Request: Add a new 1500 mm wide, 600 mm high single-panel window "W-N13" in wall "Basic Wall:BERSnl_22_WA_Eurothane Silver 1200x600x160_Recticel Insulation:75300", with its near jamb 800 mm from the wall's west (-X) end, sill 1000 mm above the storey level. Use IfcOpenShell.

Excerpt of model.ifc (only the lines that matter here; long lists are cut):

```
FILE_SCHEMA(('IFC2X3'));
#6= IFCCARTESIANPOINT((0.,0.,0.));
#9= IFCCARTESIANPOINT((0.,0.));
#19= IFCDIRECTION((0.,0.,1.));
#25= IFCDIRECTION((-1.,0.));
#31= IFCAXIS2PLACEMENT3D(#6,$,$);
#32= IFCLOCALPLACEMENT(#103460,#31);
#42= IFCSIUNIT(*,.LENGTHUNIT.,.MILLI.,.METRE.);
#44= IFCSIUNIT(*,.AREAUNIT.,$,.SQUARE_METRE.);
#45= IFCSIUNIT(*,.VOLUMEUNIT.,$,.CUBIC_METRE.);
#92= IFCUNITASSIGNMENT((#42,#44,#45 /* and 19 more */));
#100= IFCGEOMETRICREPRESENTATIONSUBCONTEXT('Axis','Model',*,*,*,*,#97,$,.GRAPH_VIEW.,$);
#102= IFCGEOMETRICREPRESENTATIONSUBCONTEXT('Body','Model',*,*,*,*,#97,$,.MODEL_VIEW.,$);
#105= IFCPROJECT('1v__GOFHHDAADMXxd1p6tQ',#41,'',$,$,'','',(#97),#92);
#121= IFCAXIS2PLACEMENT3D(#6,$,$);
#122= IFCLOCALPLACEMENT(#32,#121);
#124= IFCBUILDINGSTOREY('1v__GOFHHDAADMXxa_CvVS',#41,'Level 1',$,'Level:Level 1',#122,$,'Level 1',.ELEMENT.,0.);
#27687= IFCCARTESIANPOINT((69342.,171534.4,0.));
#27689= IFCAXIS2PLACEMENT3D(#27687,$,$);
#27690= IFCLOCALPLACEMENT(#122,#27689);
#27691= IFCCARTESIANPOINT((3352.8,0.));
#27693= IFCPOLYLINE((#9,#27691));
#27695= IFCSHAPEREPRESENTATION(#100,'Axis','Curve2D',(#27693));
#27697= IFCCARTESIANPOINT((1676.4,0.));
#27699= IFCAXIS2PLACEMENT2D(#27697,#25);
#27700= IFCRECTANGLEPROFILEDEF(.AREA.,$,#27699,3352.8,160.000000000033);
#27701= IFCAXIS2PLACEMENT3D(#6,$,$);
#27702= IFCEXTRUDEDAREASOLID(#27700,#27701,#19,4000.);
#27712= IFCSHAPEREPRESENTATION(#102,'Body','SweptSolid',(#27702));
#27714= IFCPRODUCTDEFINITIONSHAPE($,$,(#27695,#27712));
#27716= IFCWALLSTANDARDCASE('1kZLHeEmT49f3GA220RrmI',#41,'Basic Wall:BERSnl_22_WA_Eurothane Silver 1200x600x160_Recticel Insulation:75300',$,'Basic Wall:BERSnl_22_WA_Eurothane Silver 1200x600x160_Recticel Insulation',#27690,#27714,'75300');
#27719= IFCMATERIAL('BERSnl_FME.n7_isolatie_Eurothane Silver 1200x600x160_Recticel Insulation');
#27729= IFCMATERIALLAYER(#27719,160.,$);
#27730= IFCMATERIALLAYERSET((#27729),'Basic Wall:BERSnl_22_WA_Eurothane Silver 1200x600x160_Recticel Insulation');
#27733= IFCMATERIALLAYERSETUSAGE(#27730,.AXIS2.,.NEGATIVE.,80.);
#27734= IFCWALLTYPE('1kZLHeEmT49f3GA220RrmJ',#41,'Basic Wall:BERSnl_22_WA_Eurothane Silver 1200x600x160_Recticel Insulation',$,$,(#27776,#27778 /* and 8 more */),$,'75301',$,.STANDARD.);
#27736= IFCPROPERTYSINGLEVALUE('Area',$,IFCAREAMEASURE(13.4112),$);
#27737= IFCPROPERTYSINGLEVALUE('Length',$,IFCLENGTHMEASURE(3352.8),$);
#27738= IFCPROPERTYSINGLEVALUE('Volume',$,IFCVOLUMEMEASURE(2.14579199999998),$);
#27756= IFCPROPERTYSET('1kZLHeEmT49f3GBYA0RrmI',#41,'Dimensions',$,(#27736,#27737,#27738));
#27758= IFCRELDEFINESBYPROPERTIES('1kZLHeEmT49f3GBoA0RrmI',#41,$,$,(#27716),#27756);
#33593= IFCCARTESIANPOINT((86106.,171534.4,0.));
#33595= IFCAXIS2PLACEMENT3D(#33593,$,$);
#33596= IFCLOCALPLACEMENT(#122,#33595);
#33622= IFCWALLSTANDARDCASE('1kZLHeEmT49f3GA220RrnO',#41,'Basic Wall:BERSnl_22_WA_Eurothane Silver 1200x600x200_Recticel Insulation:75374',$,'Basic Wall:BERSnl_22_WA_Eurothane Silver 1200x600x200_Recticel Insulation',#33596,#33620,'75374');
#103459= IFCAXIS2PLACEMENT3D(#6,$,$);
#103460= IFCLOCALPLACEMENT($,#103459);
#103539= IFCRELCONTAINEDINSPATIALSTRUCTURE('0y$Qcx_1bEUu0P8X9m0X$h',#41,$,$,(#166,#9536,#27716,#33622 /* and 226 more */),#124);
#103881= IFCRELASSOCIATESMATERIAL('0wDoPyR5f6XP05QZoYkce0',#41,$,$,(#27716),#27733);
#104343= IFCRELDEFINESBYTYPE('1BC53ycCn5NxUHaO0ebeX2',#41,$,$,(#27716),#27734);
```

```python
import numpy as np
import ifcopenshell
import ifcopenshell.api.feature
import ifcopenshell.api.geometry
import ifcopenshell.api.pset
import ifcopenshell.api.root
import ifcopenshell.api.spatial
import ifcopenshell.api.type
import ifcopenshell.geom
import ifcopenshell.util.element
import ifcopenshell.util.placement
import ifcopenshell.util.representation
import ifcopenshell.util.shape
import ifcopenshell.util.unit

model = ifcopenshell.open("model.ifc")
unit_scale = ifcopenshell.util.unit.calculate_unit_scale(model)
area_scale = ifcopenshell.util.unit.calculate_unit_scale(model, "AREAUNIT")
volume_scale = ifcopenshell.util.unit.calculate_unit_scale(model, "VOLUMEUNIT")
settings = ifcopenshell.geom.settings()


def volume(element):
    """Net volume in cubic metres, openings subtracted."""
    shape = ifcopenshell.geom.create_shape(settings, element)
    return ifcopenshell.util.shape.get_volume(shape.geometry)


wall = model.by_guid("1kZLHeEmT49f3GA220RrmI")
storey = ifcopenshell.util.element.get_container(wall, ifc_class="IfcBuildingStorey")
context = ifcopenshell.util.representation.get_context(model, "Model", "Body", "MODEL_VIEW")
before = volume(wall)

width, height, from_end, sill = 1.5, 0.6, 0.8, 1  # metres

# The wall runs along its own X axis, and the end named is its -X end.
wall_shape = ifcopenshell.geom.create_shape(settings, wall)
x, y, z = ifcopenshell.util.shape.get_vertices(wall_shape.geometry).T
start = x.min() + from_end
face, thickness = float(y.min()), float(y.max() - y.min())
wall_matrix = ifcopenshell.util.placement.get_local_placement(wall.ObjectPlacement)
level = ifcopenshell.util.placement.get_local_placement(storey.ObjectPlacement)[2, 3]


def in_wall(x, y):
    """Placement at x, y metres in the wall's axes, at sill height."""
    matrix = wall_matrix.copy()
    matrix[:, 3] = wall_matrix @ np.array([x / unit_scale, y / unit_scale, 0.0, 1.0])
    matrix[2, 3] = level + sill / unit_scale
    return matrix


# Opening: a box that overshoots both wall faces by 50 mm.
opening = ifcopenshell.api.root.create_entity(model, ifc_class="IfcOpeningElement")
box = ifcopenshell.api.geometry.add_wall_representation(
    model, context=context, length=width, height=height, thickness=thickness + 0.1
)
ifcopenshell.api.geometry.assign_representation(model, product=opening, representation=box)
ifcopenshell.api.geometry.edit_object_placement(model, product=opening, matrix=in_wall(start, face - 0.05), is_si=False)
ifcopenshell.api.feature.add_feature(model, feature=opening, element=wall)

window = ifcopenshell.api.root.create_entity(model, ifc_class="IfcWindow", name="W-N13")
window.OverallWidth, window.OverallHeight = width / unit_scale, height / unit_scale
body = ifcopenshell.api.geometry.add_window_representation(
    model,
    context=context,
    overall_width=window.OverallWidth,
    overall_height=window.OverallHeight,
    partition_type="SINGLE_PANEL",
)
ifcopenshell.api.geometry.assign_representation(model, product=window, representation=body)
ifcopenshell.api.spatial.assign_container(model, products=[window], relating_structure=storey)
fills = ifcopenshell.api.feature.add_filling(model, opening=opening, element=window)
fills.OwnerHistory = window.OwnerHistory  # required in IFC2X3

# IFC2X3 keeps the operation on the window style.
style = ifcopenshell.api.root.create_entity(model, ifc_class="IfcWindowStyle", name="W-N13")
style.OperationType, style.ConstructionType = "SINGLE_PANEL", "NOTDEFINED"
style.ParameterTakesPrecedence = style.Sizeable = False
ifcopenshell.api.type.assign_type(model, related_objects=[window], relating_type=style)

# Centre the window in the wall's thickness.
ifcopenshell.api.geometry.edit_object_placement(model, product=window, matrix=in_wall(start, face), is_si=False)
window_shape = ifcopenshell.geom.create_shape(settings, window)
depth = ifcopenshell.util.shape.get_vertices(window_shape.geometry)[:, 1]
offset = face + thickness / 2 - (depth.min() + depth.max()) / 2
ifcopenshell.api.geometry.edit_object_placement(model, product=window, matrix=in_wall(start, offset), is_si=False)

after = volume(wall)

# Update the wall's stored quantities.
pset = model.by_id(ifcopenshell.util.element.get_pset(wall, "Dimensions", should_inherit=False)["id"])
ifcopenshell.api.pset.edit_pset(model, pset=pset, properties={
    "Area": model.create_entity("IfcAreaMeasure", after / thickness / area_scale),
    "Volume": model.create_entity("IfcVolumeMeasure", after / volume_scale),
})

print(f"wall volume {before:.3f} -> {after:.3f} m3")

model.write("model_v2.ifc")
```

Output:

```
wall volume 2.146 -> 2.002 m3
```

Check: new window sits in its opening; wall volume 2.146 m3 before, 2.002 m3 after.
